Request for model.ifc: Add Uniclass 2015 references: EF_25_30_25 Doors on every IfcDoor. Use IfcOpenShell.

First a look at what the model holds.

```python
import ifcopenshell

model = ifcopenshell.open("model.ifc")
print(model.schema)
print("classifications:", [c.Name for c in model.by_type("IfcClassification")])
for ifc_class in ("IfcDoor", "IfcRoof", "IfcStair", "IfcWall", "IfcWindow"):
    print(ifc_class, len(model.by_type(ifc_class)))
```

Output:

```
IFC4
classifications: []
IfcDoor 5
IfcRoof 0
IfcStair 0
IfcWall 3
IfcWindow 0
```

```python
import ifcopenshell
import ifcopenshell.api.classification

model = ifcopenshell.open("model.ifc")

system = ifcopenshell.api.classification.add_classification(model, classification="Uniclass 2015")

codes = {
    "IfcDoor": ("EF_25_30_25", "Doors"),
}
for ifc_class, (code, name) in codes.items():
    products = model.by_type(ifc_class)
    ifcopenshell.api.classification.add_reference(
        model, products=products, classification=system, identification=code, name=name
    )
    print(code, len(products))

model.write("model-out.ifc")
```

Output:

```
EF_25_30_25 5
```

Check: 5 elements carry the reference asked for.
